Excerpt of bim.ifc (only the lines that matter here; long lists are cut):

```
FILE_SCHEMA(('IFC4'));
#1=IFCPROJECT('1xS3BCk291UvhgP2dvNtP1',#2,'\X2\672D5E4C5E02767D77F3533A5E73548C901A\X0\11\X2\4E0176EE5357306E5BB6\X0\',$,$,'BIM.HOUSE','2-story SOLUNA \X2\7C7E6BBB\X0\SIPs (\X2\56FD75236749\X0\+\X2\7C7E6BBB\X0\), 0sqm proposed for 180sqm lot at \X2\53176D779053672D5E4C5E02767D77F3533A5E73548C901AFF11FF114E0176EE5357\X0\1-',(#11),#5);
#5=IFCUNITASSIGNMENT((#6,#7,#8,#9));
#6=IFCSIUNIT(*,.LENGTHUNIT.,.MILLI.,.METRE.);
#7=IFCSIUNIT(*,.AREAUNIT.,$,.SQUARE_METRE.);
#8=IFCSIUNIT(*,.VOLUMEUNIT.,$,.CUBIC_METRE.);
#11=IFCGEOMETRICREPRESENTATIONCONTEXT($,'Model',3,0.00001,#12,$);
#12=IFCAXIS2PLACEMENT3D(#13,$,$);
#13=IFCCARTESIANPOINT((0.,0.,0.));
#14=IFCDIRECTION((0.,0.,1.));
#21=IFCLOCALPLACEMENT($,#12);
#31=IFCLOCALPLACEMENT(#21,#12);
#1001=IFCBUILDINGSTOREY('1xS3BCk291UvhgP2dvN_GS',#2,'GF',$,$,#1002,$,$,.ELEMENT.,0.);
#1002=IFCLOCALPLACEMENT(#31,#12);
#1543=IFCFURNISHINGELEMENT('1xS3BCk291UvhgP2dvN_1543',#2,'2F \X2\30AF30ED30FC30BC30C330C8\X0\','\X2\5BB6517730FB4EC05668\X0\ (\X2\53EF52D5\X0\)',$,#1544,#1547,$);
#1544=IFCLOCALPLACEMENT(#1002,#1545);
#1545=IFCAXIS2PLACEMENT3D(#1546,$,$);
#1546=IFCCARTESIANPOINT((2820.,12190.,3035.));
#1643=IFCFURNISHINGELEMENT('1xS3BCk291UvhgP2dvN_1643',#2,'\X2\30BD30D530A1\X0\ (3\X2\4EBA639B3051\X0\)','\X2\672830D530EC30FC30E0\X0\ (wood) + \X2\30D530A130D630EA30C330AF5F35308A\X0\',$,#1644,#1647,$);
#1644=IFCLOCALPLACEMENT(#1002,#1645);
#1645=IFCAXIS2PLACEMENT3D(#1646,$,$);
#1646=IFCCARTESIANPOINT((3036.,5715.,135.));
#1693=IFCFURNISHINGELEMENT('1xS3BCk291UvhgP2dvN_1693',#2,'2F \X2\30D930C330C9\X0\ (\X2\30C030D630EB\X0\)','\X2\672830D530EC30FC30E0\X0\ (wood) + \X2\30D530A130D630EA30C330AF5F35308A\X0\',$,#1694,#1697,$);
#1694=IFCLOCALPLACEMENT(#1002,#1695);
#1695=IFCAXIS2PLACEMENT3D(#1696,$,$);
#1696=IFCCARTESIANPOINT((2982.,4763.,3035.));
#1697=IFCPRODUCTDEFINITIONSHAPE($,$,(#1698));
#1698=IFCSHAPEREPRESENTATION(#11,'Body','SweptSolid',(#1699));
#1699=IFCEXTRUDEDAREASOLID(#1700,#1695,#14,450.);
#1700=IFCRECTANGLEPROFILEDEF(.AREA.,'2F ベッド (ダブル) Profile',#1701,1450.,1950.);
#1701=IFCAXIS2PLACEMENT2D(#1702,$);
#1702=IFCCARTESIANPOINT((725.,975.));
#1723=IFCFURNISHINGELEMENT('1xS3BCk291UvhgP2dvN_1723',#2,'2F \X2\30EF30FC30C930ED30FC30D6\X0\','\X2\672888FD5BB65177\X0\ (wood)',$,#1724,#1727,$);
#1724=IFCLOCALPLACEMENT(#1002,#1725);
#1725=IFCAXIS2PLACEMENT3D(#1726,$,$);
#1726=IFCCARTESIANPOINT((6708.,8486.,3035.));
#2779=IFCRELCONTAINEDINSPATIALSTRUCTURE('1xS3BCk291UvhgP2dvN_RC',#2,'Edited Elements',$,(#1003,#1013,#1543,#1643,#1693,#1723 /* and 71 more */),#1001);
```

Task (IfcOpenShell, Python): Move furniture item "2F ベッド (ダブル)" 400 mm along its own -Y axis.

```python
import ifcopenshell
import ifcopenshell.api.geometry
import ifcopenshell.util.placement
import ifcopenshell.util.unit

model = ifcopenshell.open("bim.ifc")
unit_scale = ifcopenshell.util.unit.calculate_unit_scale(model)

item = model.by_guid("1xS3BCk291UvhgP2dvN_1693")
matrix = ifcopenshell.util.placement.get_local_placement(item.ObjectPlacement)
matrix[:3, 3] -= matrix[:3, 1] * 0.4 / unit_scale
ifcopenshell.api.geometry.edit_object_placement(model, product=item, matrix=matrix, is_si=False)

print(ifcopenshell.util.placement.get_local_placement(item.ObjectPlacement).round(3) + 0.0)

model.write("bim_v2.ifc")
```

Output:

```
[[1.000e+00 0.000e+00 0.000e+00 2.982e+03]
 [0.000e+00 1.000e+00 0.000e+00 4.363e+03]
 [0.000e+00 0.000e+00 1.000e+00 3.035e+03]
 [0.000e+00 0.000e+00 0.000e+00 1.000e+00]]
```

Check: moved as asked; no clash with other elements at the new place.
